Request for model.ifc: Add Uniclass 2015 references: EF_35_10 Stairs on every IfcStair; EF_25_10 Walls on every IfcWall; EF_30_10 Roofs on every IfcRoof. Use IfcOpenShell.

First a look at what the model holds.

```python
import ifcopenshell

model = ifcopenshell.open("model.ifc")
print(model.schema)
print("classifications:", [c.Name for c in model.by_type("IfcClassification")])
for ifc_class in ("IfcDoor", "IfcRoof", "IfcStair", "IfcWall", "IfcWindow"):
    print(ifc_class, len(model.by_type(ifc_class)))
```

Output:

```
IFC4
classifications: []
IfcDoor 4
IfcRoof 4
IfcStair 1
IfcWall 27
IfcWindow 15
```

```python
import ifcopenshell
import ifcopenshell.api.classification

model = ifcopenshell.open("model.ifc")

system = ifcopenshell.api.classification.add_classification(model, classification="Uniclass 2015")

codes = {
    "IfcStair": ("EF_35_10", "Stairs"),
    "IfcWall": ("EF_25_10", "Walls"),
    "IfcRoof": ("EF_30_10", "Roofs"),
}
for ifc_class, (code, name) in codes.items():
    products = model.by_type(ifc_class)
    ifcopenshell.api.classification.add_reference(
        model, products=products, classification=system, identification=code, name=name
    )
    print(code, len(products))

model.write("model_v2.ifc")
```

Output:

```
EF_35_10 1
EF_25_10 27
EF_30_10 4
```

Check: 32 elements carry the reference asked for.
